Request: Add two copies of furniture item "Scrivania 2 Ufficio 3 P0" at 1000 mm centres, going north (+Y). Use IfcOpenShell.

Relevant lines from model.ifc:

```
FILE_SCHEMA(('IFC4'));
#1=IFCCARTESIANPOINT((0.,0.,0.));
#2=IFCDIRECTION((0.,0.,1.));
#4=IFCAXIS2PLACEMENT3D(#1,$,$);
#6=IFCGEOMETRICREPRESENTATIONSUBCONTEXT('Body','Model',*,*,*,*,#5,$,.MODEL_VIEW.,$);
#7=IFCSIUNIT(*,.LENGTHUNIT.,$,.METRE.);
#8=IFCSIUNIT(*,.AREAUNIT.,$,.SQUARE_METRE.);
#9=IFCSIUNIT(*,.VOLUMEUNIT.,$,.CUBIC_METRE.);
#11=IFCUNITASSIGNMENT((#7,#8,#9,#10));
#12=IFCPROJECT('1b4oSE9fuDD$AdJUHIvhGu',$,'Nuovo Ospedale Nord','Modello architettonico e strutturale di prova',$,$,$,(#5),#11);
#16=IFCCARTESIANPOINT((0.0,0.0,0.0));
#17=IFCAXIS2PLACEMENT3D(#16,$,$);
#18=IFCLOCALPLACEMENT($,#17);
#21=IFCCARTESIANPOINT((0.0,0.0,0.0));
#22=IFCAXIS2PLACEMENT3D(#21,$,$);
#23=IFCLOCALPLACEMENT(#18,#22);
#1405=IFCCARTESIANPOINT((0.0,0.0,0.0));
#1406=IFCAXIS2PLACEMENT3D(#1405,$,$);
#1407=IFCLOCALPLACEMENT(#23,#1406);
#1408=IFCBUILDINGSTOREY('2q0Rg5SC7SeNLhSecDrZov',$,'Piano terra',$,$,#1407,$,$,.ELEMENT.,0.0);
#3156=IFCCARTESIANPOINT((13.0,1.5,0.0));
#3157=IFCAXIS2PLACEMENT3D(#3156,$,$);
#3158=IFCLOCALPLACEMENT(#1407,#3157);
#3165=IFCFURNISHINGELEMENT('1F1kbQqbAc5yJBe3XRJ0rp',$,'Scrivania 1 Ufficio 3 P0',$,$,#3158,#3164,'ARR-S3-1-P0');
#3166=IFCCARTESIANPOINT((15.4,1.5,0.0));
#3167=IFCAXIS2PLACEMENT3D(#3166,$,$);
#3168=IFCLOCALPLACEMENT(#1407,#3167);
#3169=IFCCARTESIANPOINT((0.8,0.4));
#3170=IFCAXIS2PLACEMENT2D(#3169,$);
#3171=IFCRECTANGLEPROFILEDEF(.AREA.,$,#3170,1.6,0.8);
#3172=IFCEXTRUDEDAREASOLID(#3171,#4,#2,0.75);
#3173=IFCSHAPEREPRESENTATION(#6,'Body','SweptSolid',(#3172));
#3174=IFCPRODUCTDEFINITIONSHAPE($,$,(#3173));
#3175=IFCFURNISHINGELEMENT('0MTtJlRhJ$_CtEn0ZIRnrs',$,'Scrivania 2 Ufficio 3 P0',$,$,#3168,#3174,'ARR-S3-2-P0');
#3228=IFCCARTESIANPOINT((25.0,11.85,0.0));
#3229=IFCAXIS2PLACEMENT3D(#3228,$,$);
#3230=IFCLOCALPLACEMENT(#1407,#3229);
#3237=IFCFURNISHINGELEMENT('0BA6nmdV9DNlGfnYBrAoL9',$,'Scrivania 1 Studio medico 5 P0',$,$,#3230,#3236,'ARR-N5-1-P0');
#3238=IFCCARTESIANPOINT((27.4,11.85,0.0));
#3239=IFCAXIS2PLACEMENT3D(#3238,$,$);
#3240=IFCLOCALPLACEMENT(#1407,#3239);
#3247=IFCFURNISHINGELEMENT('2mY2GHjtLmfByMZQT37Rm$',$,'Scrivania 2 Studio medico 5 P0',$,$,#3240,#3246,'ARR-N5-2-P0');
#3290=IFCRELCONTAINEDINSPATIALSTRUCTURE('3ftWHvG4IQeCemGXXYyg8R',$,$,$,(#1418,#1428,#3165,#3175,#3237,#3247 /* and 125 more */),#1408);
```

```python
import numpy as np
import ifcopenshell
import ifcopenshell.api.geometry
import ifcopenshell.api.root
import ifcopenshell.util.element
import ifcopenshell.util.placement
import ifcopenshell.util.unit

model = ifcopenshell.open("model.ifc")
unit_scale = ifcopenshell.util.unit.calculate_unit_scale(model)

source = model.by_guid("0MTtJlRhJ$_CtEn0ZIRnrs")
base = ifcopenshell.util.placement.get_local_placement(source.ObjectPlacement)
step = np.array([0.0, 1.0, 0.0]) * 1 / unit_scale

for i in range(1, 3):
    copy = ifcopenshell.api.root.copy_class(model, product=source)
    copy.Representation = ifcopenshell.util.element.copy_deep(
        model, source.Representation, exclude=["IfcGeometricRepresentationContext", "IfcRepresentationMap"]
    )
    copy.Tag = None
    matrix = base.copy()
    matrix[:3, 3] += i * step
    print("added at", matrix[:3, 3].round(3) + 0.0)
    ifcopenshell.api.geometry.edit_object_placement(model, product=copy, matrix=matrix, is_si=False)

model.write("model_rev.ifc")
```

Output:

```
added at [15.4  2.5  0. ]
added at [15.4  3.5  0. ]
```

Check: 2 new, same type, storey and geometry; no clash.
